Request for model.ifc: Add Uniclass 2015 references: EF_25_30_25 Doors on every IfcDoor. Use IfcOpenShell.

First a look at what the model holds.

```python
import ifcopenshell

model = ifcopenshell.open("model.ifc")
print(model.schema)
print("classifications:", [c.Name for c in model.by_type("IfcClassification")])
for ifc_class in ("IfcDoor", "IfcRoof", "IfcStair", "IfcWall", "IfcWindow"):
    print(ifc_class, len(model.by_type(ifc_class)))
```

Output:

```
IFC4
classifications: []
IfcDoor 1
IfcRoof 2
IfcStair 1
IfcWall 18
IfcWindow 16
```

```python
import ifcopenshell
import ifcopenshell.api.classification

model = ifcopenshell.open("model.ifc")

system = ifcopenshell.api.classification.add_classification(model, classification="Uniclass 2015")

codes = {
    "IfcDoor": ("EF_25_30_25", "Doors"),
}
for ifc_class, (code, name) in codes.items():
    products = model.by_type(ifc_class)
    ifcopenshell.api.classification.add_reference(
        model, products=products, classification=system, identification=code, name=name
    )
    print(code, len(products))

model.write("model_updated.ifc")
```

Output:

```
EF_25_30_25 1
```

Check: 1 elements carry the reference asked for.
